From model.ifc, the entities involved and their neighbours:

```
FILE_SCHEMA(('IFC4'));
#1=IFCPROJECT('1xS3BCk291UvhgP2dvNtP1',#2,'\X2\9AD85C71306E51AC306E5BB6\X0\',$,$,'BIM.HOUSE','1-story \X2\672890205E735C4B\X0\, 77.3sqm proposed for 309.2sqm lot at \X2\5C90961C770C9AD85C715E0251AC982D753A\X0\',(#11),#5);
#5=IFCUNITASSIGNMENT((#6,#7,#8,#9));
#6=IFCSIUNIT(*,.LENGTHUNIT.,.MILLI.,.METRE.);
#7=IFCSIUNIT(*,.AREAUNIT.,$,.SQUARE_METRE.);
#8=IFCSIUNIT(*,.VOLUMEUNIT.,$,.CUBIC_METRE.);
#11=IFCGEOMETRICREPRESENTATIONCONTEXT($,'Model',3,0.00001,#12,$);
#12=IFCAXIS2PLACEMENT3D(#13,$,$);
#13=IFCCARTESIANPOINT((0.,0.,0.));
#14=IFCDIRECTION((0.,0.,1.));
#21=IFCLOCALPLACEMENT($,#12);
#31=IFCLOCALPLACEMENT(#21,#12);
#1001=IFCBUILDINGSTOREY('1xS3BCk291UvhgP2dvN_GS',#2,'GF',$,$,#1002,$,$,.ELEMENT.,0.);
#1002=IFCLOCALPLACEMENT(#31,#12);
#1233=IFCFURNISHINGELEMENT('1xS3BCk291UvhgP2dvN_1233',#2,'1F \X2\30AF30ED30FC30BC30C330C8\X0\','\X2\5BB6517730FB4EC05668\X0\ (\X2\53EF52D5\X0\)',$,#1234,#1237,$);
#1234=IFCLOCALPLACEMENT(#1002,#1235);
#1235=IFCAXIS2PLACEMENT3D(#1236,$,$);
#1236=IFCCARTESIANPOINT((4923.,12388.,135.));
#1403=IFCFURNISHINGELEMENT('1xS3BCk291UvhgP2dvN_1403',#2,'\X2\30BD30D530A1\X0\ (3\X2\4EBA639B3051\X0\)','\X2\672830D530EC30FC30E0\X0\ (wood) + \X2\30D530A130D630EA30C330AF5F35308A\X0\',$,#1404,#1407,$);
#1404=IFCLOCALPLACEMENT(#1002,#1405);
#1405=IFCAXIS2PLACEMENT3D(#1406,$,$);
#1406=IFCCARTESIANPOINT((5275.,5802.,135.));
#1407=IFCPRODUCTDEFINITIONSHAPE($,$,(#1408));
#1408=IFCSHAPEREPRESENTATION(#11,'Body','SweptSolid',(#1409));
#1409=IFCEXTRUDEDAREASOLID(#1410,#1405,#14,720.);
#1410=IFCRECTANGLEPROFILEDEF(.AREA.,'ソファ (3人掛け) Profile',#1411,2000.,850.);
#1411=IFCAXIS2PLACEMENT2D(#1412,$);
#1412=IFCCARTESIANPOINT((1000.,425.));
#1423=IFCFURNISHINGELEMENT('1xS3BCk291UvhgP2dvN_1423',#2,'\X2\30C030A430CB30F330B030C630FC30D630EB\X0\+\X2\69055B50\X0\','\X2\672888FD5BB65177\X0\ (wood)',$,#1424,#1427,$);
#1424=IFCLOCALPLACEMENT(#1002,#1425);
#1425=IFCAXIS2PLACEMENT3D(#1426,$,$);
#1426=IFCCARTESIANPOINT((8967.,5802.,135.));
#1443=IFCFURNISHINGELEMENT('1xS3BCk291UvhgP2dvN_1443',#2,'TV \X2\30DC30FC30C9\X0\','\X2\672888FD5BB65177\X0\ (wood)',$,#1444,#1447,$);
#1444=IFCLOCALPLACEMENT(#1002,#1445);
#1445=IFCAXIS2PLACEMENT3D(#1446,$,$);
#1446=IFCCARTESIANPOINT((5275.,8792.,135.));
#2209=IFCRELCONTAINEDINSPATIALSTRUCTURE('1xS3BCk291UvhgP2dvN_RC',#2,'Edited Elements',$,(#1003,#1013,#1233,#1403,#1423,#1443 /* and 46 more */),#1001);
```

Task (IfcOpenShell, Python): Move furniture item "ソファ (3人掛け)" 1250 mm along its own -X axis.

```python
import ifcopenshell
import ifcopenshell.api.geometry
import ifcopenshell.util.placement

model = ifcopenshell.open("model.ifc")

item = model.by_guid("1xS3BCk291UvhgP2dvN_1403")
matrix = ifcopenshell.util.placement.get_local_placement(item.ObjectPlacement)
matrix[:3, 3] -= matrix[:3, 0] * 1250.0
ifcopenshell.api.geometry.edit_object_placement(model, product=item, matrix=matrix, is_si=False)

print(ifcopenshell.util.placement.get_local_placement(item.ObjectPlacement).round(3) + 0.0)

model.write("model_edited.ifc")
```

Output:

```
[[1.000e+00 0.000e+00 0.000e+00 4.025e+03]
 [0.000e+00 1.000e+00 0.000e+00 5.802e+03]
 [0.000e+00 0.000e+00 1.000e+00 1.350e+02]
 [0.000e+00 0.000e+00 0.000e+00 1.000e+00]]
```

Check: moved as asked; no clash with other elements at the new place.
